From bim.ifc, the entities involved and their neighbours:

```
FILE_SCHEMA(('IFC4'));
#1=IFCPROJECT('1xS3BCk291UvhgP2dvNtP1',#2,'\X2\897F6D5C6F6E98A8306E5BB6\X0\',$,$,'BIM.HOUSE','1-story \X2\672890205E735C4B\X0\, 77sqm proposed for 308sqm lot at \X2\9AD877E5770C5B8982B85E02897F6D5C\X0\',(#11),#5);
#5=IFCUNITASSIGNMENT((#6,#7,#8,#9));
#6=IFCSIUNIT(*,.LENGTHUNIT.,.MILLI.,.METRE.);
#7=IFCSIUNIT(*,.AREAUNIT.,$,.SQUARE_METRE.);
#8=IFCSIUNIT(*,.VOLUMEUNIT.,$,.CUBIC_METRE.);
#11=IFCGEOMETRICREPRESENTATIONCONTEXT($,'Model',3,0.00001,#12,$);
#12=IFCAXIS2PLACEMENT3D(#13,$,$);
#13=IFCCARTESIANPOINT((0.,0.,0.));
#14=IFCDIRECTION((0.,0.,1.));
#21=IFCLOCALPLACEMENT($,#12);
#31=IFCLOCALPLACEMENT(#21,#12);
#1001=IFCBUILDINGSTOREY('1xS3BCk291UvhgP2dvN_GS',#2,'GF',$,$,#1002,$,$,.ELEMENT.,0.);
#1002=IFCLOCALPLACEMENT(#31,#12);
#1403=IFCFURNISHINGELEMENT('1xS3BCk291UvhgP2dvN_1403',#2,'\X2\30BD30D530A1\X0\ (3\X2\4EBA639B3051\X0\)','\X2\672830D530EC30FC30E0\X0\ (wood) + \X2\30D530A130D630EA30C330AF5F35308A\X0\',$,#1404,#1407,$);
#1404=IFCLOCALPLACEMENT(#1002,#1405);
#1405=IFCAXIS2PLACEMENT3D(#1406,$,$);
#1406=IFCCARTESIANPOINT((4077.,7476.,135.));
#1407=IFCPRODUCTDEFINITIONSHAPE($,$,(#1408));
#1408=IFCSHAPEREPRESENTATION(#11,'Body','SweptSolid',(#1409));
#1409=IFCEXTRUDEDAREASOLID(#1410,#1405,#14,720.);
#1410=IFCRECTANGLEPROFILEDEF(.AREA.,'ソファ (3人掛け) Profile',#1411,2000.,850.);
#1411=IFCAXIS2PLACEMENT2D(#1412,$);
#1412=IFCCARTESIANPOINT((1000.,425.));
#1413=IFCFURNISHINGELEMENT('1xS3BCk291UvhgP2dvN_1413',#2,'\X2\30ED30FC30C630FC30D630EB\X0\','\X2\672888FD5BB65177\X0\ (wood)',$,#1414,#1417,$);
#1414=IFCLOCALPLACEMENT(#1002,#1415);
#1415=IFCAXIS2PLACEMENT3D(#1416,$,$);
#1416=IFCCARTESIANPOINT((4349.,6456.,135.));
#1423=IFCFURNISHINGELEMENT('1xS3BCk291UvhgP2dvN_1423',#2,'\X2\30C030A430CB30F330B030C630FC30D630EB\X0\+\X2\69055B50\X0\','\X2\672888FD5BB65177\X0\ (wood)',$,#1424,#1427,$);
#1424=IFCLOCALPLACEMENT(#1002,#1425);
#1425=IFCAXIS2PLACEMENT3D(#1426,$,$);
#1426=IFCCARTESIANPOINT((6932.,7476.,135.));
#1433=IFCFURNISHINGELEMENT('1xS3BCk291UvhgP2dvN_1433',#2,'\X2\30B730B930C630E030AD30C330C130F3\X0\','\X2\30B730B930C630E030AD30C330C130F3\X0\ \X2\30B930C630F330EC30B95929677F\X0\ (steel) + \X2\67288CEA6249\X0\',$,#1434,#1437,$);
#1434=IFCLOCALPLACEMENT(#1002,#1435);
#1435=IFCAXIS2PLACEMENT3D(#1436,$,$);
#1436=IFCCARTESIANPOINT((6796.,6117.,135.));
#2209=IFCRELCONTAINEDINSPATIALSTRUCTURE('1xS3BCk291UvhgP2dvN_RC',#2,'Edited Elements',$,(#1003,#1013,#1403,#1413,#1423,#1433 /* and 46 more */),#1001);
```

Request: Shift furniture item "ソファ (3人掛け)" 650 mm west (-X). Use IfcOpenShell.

```python
import ifcopenshell
import ifcopenshell.api.geometry
import ifcopenshell.util.placement
import ifcopenshell.util.unit

model = ifcopenshell.open("bim.ifc")
unit_scale = ifcopenshell.util.unit.calculate_unit_scale(model)

item = model.by_id(1403)
matrix = ifcopenshell.util.placement.get_local_placement(item.ObjectPlacement)
matrix[0, 3] -= 0.65 / unit_scale
ifcopenshell.api.geometry.edit_object_placement(model, product=item, matrix=matrix, is_si=False)

print(ifcopenshell.util.placement.get_local_placement(item.ObjectPlacement).round(3) + 0.0)

model.write("bim_rev.ifc")
```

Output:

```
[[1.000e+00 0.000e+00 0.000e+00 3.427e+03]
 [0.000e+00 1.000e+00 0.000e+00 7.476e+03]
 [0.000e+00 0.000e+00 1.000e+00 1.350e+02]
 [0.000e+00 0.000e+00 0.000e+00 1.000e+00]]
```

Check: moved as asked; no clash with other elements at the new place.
